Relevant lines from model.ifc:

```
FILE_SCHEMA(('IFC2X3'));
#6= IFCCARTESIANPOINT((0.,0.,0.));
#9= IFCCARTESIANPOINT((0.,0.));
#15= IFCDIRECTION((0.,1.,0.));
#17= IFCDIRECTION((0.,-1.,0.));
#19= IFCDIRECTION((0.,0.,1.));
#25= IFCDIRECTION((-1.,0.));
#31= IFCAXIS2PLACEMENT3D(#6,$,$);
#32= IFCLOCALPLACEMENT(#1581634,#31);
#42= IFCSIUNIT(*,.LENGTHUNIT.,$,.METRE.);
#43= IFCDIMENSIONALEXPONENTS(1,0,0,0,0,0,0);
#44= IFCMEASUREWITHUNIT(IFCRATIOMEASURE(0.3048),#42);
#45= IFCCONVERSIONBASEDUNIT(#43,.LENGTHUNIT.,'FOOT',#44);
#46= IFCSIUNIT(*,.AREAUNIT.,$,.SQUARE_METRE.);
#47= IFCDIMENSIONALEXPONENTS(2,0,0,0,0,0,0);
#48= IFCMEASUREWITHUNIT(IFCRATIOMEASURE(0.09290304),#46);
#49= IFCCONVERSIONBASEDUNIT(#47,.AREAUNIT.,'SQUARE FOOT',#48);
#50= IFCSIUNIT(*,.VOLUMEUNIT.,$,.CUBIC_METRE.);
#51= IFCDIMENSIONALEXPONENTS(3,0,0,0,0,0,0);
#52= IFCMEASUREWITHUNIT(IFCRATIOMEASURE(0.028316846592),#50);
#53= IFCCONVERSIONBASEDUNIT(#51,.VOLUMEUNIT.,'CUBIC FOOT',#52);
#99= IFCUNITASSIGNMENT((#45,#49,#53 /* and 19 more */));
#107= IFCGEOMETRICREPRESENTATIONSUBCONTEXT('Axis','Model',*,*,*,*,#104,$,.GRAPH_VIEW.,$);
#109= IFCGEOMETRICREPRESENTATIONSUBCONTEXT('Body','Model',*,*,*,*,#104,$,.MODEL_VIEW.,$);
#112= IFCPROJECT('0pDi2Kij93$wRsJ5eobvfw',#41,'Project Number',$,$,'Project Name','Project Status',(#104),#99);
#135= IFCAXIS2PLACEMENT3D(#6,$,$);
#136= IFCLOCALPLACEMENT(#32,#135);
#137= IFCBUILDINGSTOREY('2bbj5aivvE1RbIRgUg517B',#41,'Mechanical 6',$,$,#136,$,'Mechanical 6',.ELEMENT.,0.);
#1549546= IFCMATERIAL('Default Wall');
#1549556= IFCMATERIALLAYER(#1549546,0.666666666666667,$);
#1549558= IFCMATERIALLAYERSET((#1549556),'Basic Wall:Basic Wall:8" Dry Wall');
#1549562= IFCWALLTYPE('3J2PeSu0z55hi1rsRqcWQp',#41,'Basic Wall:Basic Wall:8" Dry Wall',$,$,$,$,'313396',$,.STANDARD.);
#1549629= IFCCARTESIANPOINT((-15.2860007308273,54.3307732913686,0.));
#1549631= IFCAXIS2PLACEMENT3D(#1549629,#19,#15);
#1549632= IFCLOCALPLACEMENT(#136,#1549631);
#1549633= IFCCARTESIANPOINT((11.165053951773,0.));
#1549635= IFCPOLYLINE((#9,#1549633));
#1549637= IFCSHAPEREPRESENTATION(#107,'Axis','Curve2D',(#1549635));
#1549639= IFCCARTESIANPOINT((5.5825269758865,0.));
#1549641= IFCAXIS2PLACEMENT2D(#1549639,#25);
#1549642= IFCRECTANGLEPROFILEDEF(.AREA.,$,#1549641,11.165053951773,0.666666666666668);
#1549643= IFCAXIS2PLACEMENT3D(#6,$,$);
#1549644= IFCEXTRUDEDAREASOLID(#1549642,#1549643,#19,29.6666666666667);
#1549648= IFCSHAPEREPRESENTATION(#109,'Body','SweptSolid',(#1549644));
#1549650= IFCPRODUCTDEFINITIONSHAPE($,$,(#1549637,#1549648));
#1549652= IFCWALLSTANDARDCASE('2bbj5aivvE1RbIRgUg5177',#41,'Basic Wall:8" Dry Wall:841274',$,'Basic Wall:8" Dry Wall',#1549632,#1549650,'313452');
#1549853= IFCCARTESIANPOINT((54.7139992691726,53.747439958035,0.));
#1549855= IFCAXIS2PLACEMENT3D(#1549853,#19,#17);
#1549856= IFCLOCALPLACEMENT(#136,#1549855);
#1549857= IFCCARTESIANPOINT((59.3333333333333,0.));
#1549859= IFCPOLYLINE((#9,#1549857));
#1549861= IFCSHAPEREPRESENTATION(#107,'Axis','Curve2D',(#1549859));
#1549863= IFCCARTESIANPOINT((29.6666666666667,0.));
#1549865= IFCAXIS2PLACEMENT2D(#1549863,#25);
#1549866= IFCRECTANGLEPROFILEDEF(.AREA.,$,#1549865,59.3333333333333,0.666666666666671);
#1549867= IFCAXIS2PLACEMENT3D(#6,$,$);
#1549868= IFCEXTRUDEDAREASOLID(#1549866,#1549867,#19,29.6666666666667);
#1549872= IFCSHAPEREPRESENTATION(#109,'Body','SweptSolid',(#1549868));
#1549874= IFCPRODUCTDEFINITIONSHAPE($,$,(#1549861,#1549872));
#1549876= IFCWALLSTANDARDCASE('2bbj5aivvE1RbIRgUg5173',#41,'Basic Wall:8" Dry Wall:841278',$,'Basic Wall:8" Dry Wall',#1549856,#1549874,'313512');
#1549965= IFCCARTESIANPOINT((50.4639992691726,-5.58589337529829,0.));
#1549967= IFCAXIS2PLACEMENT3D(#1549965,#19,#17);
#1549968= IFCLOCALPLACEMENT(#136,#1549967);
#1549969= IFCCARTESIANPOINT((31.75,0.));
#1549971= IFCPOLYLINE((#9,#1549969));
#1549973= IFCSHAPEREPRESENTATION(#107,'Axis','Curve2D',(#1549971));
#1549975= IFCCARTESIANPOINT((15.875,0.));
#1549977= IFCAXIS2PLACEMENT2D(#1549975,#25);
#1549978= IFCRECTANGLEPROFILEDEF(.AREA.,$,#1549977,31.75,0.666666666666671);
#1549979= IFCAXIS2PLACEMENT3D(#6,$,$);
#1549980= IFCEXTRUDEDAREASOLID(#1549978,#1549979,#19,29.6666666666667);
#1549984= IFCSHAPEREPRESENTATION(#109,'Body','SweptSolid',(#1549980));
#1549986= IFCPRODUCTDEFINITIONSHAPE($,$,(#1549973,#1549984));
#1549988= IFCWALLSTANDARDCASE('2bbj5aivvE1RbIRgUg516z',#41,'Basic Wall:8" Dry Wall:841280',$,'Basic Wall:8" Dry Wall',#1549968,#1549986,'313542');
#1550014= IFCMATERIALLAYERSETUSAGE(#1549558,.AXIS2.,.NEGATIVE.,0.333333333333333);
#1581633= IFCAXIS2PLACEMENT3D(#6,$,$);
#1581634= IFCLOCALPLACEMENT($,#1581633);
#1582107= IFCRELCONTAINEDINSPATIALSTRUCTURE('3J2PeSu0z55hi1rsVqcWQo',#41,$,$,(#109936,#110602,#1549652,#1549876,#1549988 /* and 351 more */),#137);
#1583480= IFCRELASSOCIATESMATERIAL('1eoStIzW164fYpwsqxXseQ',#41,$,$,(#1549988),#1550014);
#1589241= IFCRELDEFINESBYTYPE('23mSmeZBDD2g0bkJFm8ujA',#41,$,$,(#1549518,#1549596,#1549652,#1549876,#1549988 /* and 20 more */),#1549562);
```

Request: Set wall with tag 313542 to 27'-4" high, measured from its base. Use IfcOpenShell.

```python
import ifcopenshell
import ifcopenshell.geom
import ifcopenshell.util.representation
import ifcopenshell.util.shape
import ifcopenshell.util.unit

model = ifcopenshell.open("model.ifc")
unit_scale = ifcopenshell.util.unit.calculate_unit_scale(model)
settings = ifcopenshell.geom.settings()


def volume(element):
    """Net volume in cubic metres, openings subtracted."""
    shape = ifcopenshell.geom.create_shape(settings, element)
    return ifcopenshell.util.shape.get_volume(shape.geometry)


wall = model.by_guid("2bbj5aivvE1RbIRgUg516z")
before = volume(wall)

body = ifcopenshell.util.representation.get_representation(wall, "Model", "Body")
solid = body.Items[0]
old_height = solid.Depth
solid.Depth = 328 * 0.0254 / unit_scale
after = volume(wall)

print(f"height {old_height:g} -> {solid.Depth:g}, volume {before:.3f} -> {after:.3f} m3")

model.write("model_edited.ifc")
```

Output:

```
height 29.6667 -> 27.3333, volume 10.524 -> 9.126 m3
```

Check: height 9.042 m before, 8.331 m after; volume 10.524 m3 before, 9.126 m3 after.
